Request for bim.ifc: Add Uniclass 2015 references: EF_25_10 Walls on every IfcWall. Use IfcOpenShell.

First a look at what the model holds.

```python
import ifcopenshell

model = ifcopenshell.open("bim.ifc")
print(model.schema)
print("classifications:", [c.Name for c in model.by_type("IfcClassification")])
for ifc_class in ("IfcDoor", "IfcRoof", "IfcStair", "IfcWall", "IfcWindow"):
    print(ifc_class, len(model.by_type(ifc_class)))
```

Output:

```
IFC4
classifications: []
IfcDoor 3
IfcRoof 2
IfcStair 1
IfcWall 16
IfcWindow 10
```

```python
import ifcopenshell
import ifcopenshell.api.classification

model = ifcopenshell.open("bim.ifc")

system = ifcopenshell.api.classification.add_classification(model, classification="Uniclass 2015")

codes = {
    "IfcWall": ("EF_25_10", "Walls"),
}
for ifc_class, (code, name) in codes.items():
    products = model.by_type(ifc_class)
    ifcopenshell.api.classification.add_reference(
        model, products=products, classification=system, identification=code, name=name
    )
    print(code, len(products))

model.write("bim_edited.ifc")
```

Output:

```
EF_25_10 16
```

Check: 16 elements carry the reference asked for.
